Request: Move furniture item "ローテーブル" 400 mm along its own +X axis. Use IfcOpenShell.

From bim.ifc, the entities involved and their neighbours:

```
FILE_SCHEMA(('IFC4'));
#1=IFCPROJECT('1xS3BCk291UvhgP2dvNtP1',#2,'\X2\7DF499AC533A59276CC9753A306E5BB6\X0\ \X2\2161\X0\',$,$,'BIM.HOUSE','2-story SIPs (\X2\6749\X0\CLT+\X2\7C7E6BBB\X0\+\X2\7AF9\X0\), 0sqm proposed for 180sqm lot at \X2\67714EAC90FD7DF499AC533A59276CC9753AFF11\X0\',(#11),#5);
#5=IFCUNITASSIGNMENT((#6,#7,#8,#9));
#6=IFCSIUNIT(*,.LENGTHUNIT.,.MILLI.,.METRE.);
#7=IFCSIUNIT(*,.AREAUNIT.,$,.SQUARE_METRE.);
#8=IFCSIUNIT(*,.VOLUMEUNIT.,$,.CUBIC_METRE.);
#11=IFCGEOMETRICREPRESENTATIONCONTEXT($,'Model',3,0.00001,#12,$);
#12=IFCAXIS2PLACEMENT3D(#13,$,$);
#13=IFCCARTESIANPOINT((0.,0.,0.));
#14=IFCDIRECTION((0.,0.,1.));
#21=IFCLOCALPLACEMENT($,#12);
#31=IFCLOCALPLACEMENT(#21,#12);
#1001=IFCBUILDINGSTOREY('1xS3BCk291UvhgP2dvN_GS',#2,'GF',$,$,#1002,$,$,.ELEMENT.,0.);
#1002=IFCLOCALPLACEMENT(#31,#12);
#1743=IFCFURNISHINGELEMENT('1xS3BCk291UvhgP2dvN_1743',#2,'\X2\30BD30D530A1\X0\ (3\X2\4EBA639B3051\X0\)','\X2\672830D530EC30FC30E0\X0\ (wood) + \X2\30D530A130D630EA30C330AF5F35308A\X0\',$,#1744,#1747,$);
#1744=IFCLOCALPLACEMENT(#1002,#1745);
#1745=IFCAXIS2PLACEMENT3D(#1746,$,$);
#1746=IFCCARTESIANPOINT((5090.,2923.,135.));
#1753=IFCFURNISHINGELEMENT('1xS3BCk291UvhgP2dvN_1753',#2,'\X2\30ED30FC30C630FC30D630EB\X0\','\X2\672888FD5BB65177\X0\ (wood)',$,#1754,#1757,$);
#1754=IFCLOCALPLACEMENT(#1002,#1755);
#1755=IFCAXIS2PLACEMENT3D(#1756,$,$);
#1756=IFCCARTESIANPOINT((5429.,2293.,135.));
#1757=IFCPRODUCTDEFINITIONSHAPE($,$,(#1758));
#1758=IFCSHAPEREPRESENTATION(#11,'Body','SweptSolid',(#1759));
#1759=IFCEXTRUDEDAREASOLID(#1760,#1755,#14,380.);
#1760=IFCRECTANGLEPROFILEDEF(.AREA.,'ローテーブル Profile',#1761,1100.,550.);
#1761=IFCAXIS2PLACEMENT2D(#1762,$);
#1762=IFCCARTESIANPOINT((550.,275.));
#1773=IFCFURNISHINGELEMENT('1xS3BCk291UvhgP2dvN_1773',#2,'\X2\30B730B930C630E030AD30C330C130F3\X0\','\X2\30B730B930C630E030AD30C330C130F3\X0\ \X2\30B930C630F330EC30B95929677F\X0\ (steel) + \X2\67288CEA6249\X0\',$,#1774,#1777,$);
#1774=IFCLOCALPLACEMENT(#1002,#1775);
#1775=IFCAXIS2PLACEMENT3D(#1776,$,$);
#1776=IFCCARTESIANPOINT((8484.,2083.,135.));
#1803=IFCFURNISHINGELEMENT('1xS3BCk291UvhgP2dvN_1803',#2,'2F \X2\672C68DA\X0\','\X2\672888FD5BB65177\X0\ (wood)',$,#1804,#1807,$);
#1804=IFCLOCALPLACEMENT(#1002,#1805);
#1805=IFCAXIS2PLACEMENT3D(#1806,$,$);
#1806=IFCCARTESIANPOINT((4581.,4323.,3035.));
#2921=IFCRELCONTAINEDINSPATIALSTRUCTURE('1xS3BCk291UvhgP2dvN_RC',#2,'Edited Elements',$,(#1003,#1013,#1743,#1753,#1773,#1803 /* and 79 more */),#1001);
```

```python
import ifcopenshell
import ifcopenshell.api.geometry
import ifcopenshell.util.placement

model = ifcopenshell.open("bim.ifc")

item = model.by_guid("1xS3BCk291UvhgP2dvN_1753")
matrix = ifcopenshell.util.placement.get_local_placement(item.ObjectPlacement)
matrix[:3, 3] += matrix[:3, 0] * 400.0
ifcopenshell.api.geometry.edit_object_placement(model, product=item, matrix=matrix, is_si=False)

print(ifcopenshell.util.placement.get_local_placement(item.ObjectPlacement).round(3) + 0.0)

model.write("bim_edited.ifc")
```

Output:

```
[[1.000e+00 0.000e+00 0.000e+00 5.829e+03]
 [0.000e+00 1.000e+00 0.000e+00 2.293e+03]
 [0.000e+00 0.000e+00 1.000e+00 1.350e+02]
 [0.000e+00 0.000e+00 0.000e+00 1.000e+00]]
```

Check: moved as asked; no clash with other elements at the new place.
